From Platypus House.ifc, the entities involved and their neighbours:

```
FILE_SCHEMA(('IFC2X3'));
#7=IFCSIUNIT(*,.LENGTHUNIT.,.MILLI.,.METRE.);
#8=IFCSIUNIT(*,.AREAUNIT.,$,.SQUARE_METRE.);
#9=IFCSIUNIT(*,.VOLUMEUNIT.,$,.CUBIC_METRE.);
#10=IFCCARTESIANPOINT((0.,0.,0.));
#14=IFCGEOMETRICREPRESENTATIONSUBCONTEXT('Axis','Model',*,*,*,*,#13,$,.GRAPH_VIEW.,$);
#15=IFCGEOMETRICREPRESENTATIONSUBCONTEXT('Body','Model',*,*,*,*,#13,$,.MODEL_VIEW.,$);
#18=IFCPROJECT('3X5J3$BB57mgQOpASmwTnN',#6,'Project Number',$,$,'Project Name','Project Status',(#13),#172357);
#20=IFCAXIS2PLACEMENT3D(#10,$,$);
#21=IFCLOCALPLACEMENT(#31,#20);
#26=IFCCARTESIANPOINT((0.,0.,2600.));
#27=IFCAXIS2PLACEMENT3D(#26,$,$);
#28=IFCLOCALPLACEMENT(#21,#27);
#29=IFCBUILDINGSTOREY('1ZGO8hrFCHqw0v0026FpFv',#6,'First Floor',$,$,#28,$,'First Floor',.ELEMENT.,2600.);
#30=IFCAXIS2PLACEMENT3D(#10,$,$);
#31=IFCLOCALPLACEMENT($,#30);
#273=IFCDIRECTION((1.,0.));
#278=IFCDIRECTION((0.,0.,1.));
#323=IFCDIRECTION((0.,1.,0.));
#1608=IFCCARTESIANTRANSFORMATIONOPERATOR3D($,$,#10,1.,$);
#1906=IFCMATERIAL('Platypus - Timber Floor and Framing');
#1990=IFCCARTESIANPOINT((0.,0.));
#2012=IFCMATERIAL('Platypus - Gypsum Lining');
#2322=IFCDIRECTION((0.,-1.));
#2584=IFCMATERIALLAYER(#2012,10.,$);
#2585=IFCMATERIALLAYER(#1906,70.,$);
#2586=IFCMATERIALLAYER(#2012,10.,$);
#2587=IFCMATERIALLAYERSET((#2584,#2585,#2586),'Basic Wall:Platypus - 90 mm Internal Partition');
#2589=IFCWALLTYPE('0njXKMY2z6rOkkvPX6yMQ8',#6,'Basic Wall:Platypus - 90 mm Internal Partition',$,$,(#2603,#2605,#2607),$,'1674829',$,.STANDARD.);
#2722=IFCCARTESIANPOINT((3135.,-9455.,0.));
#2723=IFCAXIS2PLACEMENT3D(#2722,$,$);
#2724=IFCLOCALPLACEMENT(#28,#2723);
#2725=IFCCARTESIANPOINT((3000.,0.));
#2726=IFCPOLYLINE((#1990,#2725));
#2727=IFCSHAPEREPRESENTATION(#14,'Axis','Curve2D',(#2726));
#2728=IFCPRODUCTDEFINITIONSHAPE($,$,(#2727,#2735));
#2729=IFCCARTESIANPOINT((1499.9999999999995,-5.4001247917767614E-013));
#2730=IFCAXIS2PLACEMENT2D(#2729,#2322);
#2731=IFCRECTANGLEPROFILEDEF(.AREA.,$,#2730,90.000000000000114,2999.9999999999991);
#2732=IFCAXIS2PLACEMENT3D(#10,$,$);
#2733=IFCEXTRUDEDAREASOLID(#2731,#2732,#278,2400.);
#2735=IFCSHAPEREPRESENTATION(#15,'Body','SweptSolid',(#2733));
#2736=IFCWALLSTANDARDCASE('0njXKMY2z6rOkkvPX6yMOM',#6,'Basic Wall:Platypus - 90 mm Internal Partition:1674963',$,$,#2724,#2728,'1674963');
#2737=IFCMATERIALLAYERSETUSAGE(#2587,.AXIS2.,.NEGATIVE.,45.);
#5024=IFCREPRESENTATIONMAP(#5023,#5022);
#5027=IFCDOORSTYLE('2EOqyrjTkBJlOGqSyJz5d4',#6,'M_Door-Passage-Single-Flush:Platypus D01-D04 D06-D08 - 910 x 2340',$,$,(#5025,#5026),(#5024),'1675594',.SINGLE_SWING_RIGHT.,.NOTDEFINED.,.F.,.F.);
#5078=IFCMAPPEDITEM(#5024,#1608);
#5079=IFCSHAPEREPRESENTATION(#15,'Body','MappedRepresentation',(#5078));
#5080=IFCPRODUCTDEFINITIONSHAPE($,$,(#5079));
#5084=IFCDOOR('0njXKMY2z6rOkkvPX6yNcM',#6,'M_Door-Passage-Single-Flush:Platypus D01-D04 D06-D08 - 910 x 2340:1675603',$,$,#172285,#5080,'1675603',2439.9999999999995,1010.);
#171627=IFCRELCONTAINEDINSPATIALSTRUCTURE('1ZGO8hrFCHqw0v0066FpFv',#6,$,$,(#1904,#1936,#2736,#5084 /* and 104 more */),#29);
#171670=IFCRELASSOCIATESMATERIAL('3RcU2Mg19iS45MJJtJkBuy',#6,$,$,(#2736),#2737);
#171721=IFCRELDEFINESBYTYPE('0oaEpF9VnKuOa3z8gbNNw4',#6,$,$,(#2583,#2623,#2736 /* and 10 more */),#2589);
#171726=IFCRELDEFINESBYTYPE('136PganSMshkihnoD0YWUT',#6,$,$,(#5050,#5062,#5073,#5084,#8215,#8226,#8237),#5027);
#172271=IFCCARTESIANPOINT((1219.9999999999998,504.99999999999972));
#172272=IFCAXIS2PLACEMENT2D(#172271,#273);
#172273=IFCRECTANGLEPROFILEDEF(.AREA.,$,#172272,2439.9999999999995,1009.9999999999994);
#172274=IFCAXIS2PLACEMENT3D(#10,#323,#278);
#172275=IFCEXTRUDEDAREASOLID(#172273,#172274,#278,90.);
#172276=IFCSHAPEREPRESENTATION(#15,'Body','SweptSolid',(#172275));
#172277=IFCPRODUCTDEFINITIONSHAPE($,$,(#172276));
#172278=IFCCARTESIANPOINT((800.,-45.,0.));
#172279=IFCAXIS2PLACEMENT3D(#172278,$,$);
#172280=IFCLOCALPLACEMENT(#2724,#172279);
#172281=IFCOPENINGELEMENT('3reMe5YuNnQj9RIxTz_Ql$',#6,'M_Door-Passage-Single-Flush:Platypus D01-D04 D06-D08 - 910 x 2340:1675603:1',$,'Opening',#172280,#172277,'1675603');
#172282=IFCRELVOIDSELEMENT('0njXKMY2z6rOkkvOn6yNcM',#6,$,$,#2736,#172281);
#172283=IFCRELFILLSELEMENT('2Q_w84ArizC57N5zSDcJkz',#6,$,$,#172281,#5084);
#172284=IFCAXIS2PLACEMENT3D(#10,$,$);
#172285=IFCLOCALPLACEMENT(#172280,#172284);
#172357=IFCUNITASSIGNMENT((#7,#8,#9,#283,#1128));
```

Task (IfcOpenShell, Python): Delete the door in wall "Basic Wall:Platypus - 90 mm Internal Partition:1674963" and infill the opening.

```python
import ifcopenshell
import ifcopenshell.api.feature
import ifcopenshell.api.root
import ifcopenshell.geom
import ifcopenshell.util.shape

model = ifcopenshell.open("Platypus House.ifc")
settings = ifcopenshell.geom.settings()


def volume(element):
    """Net volume in cubic metres, openings subtracted."""
    shape = ifcopenshell.geom.create_shape(settings, element)
    return ifcopenshell.util.shape.get_volume(shape.geometry)


door = model.by_id(5084)
opening = door.FillsVoids[0].RelatingOpeningElement
wall = opening.VoidsElements[0].RelatingBuildingElement
before = volume(wall)

ifcopenshell.api.root.remove_product(model, product=door)
ifcopenshell.api.feature.remove_feature(model, feature=opening)

after = volume(wall)

print(f"wall volume {before:.3f} -> {after:.3f} m3")

model.write("Platypus House_edited.ifc")
```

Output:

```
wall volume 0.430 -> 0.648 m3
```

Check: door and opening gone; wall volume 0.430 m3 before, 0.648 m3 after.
